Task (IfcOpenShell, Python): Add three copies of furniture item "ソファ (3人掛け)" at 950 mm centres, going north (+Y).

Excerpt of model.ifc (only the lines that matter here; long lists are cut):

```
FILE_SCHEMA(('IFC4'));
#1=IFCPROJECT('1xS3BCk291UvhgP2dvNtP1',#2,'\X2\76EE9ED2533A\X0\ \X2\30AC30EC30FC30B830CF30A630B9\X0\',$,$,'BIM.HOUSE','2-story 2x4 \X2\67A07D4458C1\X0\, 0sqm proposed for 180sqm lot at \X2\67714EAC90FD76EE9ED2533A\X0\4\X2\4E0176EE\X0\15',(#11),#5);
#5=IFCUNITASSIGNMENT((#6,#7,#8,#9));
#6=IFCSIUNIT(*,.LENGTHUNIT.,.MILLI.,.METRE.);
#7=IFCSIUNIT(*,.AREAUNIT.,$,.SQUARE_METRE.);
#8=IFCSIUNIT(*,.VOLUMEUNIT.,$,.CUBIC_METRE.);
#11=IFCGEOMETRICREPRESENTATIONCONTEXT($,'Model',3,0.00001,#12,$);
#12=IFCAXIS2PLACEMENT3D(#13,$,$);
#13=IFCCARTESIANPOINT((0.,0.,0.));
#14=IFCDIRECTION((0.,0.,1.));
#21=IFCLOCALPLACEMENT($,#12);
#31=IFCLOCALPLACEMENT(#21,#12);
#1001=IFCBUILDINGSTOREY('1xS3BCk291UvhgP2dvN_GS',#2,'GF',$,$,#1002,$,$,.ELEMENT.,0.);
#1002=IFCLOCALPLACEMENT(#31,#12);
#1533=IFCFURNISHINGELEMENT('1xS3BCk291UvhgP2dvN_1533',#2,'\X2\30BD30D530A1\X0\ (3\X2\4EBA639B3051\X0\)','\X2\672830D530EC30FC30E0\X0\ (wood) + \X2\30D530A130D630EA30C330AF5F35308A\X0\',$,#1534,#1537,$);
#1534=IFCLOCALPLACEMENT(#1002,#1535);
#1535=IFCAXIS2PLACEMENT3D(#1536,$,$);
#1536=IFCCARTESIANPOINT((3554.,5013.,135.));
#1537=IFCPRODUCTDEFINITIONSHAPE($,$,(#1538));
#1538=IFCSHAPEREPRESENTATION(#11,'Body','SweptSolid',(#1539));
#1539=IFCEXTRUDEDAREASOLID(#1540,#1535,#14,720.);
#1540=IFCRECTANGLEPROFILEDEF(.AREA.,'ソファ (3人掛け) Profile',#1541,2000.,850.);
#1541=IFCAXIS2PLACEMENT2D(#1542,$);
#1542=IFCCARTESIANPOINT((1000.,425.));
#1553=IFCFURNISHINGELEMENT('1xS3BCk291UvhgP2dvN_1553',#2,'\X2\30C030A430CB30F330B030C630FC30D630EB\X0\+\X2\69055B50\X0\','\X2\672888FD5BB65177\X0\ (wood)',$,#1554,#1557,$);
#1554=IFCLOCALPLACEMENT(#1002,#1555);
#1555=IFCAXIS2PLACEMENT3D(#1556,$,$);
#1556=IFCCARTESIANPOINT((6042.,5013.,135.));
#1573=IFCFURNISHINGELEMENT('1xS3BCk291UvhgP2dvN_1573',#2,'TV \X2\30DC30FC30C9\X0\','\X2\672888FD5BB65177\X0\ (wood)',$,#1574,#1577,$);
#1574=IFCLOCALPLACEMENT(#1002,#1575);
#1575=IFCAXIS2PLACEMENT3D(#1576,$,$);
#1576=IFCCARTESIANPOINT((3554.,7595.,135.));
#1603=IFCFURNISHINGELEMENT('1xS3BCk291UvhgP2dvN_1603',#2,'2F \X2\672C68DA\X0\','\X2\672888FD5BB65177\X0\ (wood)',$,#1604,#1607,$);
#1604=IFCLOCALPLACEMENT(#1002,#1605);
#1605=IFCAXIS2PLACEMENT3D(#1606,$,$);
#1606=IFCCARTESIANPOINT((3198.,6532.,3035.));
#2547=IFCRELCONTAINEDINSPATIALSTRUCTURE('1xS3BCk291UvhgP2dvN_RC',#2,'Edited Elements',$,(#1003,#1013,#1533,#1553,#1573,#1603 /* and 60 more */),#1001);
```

```python
import numpy as np
import ifcopenshell
import ifcopenshell.api.geometry
import ifcopenshell.api.root
import ifcopenshell.util.element
import ifcopenshell.util.placement
import ifcopenshell.util.unit

model = ifcopenshell.open("model.ifc")
unit_scale = ifcopenshell.util.unit.calculate_unit_scale(model)


def reuse_history(source, copy):
    """copy_class also copies each property set's owner history, people and application; keep the originals."""
    for rel in copy.IsDefinedBy:
        if rel.is_a("IfcRelDefinesByProperties") and (history := rel.RelatingPropertyDefinition.OwnerHistory):
            rel.RelatingPropertyDefinition.OwnerHistory = source.OwnerHistory
            ifcopenshell.util.element.remove_deep2(model, history)


source = model.by_guid("1xS3BCk291UvhgP2dvN_1533")
base = ifcopenshell.util.placement.get_local_placement(source.ObjectPlacement)
step = np.array([0.0, 1.0, 0.0]) * 0.95 / unit_scale

for i in range(1, 4):
    copy = ifcopenshell.api.root.copy_class(model, product=source)
    copy.Representation = ifcopenshell.util.element.copy_deep(
        model, source.Representation, exclude=["IfcGeometricRepresentationContext", "IfcRepresentationMap"]
    )
    reuse_history(source, copy)
    matrix = base.copy()
    matrix[:3, 3] += i * step
    print("added at", matrix[:3, 3].round(3) + 0.0)
    ifcopenshell.api.geometry.edit_object_placement(model, product=copy, matrix=matrix, is_si=False)

model.write("model_edited.ifc")
```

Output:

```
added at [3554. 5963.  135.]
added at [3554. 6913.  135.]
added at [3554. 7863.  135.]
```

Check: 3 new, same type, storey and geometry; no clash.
